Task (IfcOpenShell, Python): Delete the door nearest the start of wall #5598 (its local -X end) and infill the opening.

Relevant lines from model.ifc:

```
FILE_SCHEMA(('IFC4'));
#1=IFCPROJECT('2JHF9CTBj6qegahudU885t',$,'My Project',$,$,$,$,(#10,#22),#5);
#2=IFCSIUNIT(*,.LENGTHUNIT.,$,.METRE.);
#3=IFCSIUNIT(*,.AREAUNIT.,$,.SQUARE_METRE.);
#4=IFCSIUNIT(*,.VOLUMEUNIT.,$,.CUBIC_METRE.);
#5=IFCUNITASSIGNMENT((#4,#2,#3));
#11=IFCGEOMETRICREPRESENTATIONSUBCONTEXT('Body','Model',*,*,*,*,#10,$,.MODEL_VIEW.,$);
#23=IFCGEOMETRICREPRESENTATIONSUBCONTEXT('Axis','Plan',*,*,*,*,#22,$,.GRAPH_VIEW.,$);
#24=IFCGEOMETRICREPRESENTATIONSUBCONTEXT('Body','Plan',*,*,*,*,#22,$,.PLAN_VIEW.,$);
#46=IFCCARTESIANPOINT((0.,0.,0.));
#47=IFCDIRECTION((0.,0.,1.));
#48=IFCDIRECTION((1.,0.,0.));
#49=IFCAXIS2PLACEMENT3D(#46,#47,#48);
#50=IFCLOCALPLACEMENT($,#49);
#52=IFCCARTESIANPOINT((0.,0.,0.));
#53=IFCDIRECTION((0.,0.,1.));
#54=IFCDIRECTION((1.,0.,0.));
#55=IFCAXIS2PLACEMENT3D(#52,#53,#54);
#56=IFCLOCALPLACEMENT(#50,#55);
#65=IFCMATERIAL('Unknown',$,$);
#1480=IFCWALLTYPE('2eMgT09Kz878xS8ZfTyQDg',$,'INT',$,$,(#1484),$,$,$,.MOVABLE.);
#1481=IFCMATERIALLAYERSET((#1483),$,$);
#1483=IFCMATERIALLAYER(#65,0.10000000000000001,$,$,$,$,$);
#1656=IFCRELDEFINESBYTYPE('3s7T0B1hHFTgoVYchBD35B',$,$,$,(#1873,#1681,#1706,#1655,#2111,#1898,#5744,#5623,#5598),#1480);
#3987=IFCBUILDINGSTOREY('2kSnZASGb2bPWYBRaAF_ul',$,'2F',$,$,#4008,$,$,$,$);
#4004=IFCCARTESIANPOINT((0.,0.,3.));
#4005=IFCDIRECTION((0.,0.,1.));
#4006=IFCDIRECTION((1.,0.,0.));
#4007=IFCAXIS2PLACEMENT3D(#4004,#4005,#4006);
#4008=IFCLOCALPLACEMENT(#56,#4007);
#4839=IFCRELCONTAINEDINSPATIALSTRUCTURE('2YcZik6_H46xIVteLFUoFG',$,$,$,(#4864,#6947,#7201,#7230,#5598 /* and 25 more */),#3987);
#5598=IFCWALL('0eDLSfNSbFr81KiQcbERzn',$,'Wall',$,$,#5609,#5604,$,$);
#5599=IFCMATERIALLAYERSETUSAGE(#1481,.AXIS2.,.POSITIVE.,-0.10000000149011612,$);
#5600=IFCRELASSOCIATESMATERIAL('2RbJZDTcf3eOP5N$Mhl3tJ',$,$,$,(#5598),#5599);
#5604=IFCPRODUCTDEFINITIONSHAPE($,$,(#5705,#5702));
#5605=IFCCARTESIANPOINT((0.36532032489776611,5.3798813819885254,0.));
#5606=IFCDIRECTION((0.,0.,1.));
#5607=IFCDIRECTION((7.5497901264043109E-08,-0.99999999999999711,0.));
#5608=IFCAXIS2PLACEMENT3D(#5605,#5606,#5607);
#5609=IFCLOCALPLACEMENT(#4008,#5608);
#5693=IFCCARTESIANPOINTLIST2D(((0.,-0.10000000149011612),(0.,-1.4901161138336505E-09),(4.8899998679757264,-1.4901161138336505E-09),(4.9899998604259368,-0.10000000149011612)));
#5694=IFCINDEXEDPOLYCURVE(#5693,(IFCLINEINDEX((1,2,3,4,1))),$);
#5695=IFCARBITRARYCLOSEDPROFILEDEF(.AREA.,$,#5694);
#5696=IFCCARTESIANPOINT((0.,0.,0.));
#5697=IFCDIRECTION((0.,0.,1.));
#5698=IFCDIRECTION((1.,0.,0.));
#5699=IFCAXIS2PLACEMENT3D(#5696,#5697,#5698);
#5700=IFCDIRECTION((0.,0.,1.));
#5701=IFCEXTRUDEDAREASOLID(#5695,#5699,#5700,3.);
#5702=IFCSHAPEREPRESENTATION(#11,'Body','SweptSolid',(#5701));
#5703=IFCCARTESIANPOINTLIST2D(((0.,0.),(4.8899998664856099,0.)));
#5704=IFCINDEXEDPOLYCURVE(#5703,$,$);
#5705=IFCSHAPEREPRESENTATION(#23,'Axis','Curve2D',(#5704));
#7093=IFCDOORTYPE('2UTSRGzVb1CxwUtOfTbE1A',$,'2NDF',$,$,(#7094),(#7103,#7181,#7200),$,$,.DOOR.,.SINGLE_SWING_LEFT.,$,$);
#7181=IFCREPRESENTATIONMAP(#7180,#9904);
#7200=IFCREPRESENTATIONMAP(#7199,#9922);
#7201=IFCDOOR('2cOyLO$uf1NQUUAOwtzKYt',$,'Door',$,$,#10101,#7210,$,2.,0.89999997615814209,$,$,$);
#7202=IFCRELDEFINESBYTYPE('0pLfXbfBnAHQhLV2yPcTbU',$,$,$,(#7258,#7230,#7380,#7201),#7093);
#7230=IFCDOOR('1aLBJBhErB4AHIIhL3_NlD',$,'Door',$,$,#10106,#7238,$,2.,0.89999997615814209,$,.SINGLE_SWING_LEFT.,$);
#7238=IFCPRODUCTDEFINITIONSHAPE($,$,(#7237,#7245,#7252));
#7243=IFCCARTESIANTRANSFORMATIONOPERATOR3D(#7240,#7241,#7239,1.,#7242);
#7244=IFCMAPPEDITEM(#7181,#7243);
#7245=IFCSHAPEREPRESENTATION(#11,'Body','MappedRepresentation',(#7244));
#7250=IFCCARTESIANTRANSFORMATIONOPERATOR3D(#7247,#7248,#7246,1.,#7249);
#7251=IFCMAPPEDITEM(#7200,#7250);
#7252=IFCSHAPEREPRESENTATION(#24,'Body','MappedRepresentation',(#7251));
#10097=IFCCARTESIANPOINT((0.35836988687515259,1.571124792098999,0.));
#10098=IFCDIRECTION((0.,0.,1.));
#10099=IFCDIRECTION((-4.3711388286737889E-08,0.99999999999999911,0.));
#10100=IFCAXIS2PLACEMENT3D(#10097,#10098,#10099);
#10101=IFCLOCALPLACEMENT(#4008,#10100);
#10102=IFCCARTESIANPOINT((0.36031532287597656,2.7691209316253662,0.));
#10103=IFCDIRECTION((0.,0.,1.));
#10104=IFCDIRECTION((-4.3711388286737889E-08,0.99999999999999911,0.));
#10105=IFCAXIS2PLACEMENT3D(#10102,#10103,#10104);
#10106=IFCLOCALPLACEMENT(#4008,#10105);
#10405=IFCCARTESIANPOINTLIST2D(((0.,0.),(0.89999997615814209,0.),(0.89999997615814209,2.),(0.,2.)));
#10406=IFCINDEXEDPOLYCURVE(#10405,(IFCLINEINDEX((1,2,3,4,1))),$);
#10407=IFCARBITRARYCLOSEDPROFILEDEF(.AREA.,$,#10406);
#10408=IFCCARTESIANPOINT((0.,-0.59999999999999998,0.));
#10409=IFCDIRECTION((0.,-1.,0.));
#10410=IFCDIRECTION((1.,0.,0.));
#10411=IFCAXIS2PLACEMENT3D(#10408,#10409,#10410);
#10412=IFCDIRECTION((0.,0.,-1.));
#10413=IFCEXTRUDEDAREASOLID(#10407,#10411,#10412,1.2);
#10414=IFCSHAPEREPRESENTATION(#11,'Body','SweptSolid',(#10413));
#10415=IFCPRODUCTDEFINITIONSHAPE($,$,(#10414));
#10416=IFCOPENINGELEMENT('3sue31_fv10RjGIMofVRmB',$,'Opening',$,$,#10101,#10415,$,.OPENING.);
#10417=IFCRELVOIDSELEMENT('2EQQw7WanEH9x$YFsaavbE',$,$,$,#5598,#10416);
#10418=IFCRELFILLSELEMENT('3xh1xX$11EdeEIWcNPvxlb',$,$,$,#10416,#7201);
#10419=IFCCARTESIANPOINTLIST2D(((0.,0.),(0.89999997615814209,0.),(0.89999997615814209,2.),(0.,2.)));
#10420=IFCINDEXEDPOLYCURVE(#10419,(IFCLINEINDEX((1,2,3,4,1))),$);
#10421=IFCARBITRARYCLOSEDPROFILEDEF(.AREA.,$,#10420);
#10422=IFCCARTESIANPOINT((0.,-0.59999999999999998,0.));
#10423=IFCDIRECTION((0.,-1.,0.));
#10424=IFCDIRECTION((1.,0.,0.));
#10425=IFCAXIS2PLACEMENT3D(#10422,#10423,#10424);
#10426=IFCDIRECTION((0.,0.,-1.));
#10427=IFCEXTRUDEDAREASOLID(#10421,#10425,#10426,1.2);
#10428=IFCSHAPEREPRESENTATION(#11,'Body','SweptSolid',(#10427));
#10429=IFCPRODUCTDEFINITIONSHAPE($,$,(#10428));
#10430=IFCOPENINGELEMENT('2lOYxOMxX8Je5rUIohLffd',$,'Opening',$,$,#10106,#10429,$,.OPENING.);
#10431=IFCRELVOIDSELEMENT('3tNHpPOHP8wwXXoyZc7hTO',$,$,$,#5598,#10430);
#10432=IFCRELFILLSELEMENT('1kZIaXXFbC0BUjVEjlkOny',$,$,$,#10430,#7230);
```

```python
import ifcopenshell
import ifcopenshell.api.feature
import ifcopenshell.api.root
import ifcopenshell.geom
import ifcopenshell.util.shape

model = ifcopenshell.open("model.ifc")
settings = ifcopenshell.geom.settings()


def volume(element):
    """Net volume in cubic metres, openings subtracted."""
    shape = ifcopenshell.geom.create_shape(settings, element)
    return ifcopenshell.util.shape.get_volume(shape.geometry)


door = model.by_guid("1aLBJBhErB4AHIIhL3_NlD")
opening = door.FillsVoids[0].RelatingOpeningElement
wall = opening.VoidsElements[0].RelatingBuildingElement
before = volume(wall)

ifcopenshell.api.root.remove_product(model, product=door)
ifcopenshell.api.feature.remove_feature(model, feature=opening)

after = volume(wall)

print(f"wall volume {before:.3f} -> {after:.3f} m3")

model.write("model_updated.ifc")
```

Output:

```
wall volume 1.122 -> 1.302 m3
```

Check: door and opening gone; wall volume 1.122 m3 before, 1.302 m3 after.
